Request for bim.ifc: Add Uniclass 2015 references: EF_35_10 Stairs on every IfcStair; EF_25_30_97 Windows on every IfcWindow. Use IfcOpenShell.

First a look at what the model holds.

```python
import ifcopenshell

model = ifcopenshell.open("bim.ifc")
print(model.schema)
print("classifications:", [c.Name for c in model.by_type("IfcClassification")])
for ifc_class in ("IfcDoor", "IfcRoof", "IfcStair", "IfcWall", "IfcWindow"):
    print(ifc_class, len(model.by_type(ifc_class)))
```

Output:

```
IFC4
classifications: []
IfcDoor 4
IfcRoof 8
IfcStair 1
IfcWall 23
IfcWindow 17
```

```python
import ifcopenshell
import ifcopenshell.api.classification

model = ifcopenshell.open("bim.ifc")

system = ifcopenshell.api.classification.add_classification(model, classification="Uniclass 2015")

codes = {
    "IfcStair": ("EF_35_10", "Stairs"),
    "IfcWindow": ("EF_25_30_97", "Windows"),
}
for ifc_class, (code, name) in codes.items():
    products = model.by_type(ifc_class)
    ifcopenshell.api.classification.add_reference(
        model, products=products, classification=system, identification=code, name=name
    )
    print(code, len(products))

model.write("bim-out.ifc")
```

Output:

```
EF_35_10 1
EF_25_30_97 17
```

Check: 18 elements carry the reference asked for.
